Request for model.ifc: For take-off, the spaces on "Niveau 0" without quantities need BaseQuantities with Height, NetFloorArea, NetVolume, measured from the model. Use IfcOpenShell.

First a look at what the model holds.

```python
import ifcopenshell
import ifcopenshell.util.element
import ifcopenshell.util.unit

model = ifcopenshell.open("model.ifc")
print(model.schema)
for unit_type in ("LENGTHUNIT", "AREAUNIT", "VOLUMEUNIT"):
    print(unit_type, ifcopenshell.util.unit.calculate_unit_scale(model, unit_type))
storey = next(s for s in model.by_type("IfcBuildingStorey") if s.Name == "Niveau 0")
spaces = [e for e in ifcopenshell.util.element.get_decomposition(storey) if e.is_a("IfcSpace")]
for e in sorted(spaces, key=lambda e: e.id()):
    print(e.id(), e.is_a(), e.Name, list(ifcopenshell.util.element.get_psets(e, qtos_only=True)), sep=" | ")
```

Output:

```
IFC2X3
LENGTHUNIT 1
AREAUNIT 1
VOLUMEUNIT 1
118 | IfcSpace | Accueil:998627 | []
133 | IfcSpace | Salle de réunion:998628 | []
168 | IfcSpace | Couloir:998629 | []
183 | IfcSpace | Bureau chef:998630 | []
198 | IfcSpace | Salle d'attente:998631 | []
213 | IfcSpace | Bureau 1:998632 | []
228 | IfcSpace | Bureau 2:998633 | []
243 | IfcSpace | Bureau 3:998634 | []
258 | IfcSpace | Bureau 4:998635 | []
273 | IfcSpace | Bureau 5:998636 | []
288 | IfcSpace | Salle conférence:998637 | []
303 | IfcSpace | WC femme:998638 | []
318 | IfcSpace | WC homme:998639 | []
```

```python
import ifcopenshell
import ifcopenshell.api.pset
import ifcopenshell.geom
import ifcopenshell.util.element
import ifcopenshell.util.shape
import ifcopenshell.util.unit

model = ifcopenshell.open("model.ifc")
unit_scale = ifcopenshell.util.unit.calculate_unit_scale(model)
area_scale = ifcopenshell.util.unit.calculate_unit_scale(model, "AREAUNIT")
volume_scale = ifcopenshell.util.unit.calculate_unit_scale(model, "VOLUMEUNIT")
settings = ifcopenshell.geom.settings()

storey = next(s for s in model.by_type("IfcBuildingStorey") if s.Name == "Niveau 0")
spaces = [e for e in ifcopenshell.util.element.get_decomposition(storey) if e.is_a("IfcSpace")]

for e in sorted(spaces, key=lambda e: e.id()):
    if ifcopenshell.util.element.get_psets(e, qtos_only=True, should_inherit=False):
        continue
    # Geometry comes back in metres, in the element's own axes.
    shape = ifcopenshell.geom.create_shape(settings, e)
    values = {
        "Height": ifcopenshell.util.shape.get_z(shape.geometry) / unit_scale,
        "NetFloorArea": ifcopenshell.util.shape.get_footprint_area(shape.geometry) / area_scale,
        "NetVolume": ifcopenshell.util.shape.get_volume(shape.geometry) / volume_scale,
    }
    qto = ifcopenshell.api.pset.add_qto(model, product=e, name="BaseQuantities")
    ifcopenshell.api.pset.edit_qto(model, qto=qto, properties=values)
    print(e.id(), {k: round(v, 3) for k, v in values.items()})

model.write("model_rev.ifc")
```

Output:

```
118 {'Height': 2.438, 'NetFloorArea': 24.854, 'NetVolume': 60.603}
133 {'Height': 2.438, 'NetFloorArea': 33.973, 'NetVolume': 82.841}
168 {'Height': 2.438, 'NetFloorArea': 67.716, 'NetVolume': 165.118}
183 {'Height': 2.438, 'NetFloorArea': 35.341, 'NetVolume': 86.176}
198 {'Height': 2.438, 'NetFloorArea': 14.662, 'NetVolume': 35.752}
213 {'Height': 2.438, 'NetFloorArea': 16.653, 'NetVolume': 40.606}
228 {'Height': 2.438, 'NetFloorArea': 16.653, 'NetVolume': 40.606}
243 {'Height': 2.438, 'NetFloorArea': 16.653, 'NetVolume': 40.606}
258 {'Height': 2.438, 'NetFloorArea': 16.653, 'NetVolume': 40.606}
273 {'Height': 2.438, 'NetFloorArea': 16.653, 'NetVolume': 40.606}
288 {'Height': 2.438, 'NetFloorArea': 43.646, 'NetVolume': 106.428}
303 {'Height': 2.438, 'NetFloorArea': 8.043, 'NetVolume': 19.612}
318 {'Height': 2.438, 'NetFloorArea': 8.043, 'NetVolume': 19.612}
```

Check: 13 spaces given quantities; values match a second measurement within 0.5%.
